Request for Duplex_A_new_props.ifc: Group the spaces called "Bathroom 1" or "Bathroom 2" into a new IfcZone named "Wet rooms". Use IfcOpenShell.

First a look at what the model holds.

```python
import ifcopenshell

model = ifcopenshell.open("Duplex_A_new_props.ifc")
print(model.schema)
seen = {}
for space in model.by_type("IfcSpace"):
    seen[space.LongName] = seen.get(space.LongName, 0) + 1
for name, count in sorted(seen.items(), key=str):
    print(count, "x", name)
print("zones:", [z.Name for z in model.by_type("IfcZone")][:20])
```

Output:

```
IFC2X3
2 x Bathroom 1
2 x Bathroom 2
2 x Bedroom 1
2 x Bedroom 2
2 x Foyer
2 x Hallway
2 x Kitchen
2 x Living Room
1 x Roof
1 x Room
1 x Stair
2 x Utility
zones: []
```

```python
import ifcopenshell
import ifcopenshell.api.group
import ifcopenshell.api.root

model = ifcopenshell.open("Duplex_A_new_props.ifc")

names = {"Bathroom 1", "Bathroom 2"}
spaces = [s for s in model.by_type("IfcSpace") if s.LongName in names]

zone = ifcopenshell.api.root.create_entity(model, ifc_class="IfcZone", name="Wet rooms")
ifcopenshell.api.group.assign_group(model, products=spaces, group=zone)
print(len(spaces), "spaces in", zone.Name)

model.write("Duplex_A_new_props_v2.ifc")
```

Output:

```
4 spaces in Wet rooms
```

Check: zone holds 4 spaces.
